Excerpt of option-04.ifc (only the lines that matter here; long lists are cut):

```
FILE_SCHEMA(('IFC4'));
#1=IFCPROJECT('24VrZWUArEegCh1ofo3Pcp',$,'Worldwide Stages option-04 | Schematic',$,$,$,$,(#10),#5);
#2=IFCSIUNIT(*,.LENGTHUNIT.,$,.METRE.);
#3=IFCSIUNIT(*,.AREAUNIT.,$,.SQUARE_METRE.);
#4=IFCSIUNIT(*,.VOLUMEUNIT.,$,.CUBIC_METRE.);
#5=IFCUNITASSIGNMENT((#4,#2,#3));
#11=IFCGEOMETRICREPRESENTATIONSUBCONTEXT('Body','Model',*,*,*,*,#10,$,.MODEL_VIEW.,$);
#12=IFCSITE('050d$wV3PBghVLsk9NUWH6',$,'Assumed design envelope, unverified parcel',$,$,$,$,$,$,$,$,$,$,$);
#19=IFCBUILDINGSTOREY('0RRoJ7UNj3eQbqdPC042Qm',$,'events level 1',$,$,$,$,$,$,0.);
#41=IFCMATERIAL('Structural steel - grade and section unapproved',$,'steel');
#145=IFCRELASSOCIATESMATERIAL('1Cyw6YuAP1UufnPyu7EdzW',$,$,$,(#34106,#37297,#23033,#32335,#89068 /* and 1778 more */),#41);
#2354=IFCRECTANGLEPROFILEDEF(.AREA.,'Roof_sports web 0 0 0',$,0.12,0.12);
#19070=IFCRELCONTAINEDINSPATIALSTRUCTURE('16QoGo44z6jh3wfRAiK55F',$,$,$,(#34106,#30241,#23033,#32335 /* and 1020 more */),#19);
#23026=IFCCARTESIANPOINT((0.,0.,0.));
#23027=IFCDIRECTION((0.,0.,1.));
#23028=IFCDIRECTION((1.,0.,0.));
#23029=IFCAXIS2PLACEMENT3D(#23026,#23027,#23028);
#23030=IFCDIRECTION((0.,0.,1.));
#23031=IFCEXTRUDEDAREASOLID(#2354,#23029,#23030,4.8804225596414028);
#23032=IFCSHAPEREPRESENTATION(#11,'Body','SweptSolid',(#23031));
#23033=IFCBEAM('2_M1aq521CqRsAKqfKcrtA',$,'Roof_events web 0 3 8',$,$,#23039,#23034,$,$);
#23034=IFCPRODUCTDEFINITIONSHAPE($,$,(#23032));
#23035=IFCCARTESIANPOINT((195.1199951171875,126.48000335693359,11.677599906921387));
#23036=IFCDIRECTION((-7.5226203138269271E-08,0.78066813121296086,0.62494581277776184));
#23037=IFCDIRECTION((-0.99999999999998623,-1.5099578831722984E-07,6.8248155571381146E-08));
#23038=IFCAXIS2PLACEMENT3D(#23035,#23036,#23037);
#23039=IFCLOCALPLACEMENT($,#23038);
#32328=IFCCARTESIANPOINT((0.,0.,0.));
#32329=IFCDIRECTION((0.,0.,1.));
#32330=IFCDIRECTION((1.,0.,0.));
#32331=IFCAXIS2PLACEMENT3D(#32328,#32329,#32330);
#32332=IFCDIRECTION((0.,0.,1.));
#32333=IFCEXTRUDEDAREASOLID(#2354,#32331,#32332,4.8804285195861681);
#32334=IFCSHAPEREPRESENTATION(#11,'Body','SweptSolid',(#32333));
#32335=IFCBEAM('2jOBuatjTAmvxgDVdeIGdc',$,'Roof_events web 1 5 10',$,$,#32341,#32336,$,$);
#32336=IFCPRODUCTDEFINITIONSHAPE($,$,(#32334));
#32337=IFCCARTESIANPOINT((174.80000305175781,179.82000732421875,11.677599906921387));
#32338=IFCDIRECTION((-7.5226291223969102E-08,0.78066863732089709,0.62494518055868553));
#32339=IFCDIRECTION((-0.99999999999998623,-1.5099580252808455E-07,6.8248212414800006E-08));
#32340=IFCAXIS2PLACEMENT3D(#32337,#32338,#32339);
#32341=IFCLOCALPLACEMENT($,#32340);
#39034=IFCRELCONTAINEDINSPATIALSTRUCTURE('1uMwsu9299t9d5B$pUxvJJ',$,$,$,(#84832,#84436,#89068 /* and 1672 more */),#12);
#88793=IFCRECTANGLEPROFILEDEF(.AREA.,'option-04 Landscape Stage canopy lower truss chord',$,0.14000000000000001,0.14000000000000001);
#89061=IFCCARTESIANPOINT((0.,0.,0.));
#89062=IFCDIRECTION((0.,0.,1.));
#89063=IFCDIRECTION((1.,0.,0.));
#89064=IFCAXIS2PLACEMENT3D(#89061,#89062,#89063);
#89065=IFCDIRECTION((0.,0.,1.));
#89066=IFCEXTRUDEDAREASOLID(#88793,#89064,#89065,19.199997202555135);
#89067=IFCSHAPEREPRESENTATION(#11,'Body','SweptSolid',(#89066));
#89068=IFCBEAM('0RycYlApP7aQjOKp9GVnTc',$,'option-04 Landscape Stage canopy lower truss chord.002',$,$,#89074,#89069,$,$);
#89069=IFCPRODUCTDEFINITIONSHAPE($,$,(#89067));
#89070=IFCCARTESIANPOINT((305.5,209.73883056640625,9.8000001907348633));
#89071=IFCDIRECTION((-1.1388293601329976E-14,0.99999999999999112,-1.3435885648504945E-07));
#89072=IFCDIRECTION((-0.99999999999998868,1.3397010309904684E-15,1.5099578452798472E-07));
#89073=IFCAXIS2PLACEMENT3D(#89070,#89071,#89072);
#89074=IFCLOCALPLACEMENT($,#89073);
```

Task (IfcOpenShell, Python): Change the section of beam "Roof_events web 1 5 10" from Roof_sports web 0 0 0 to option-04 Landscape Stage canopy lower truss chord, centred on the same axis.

```python
import ifcopenshell
import ifcopenshell.util.element
import ifcopenshell.util.representation

model = ifcopenshell.open("option-04.ifc")

member = model.by_id(32335)
source = next(p for p in model.by_type("IfcRectangleProfileDef") if p.ProfileName == "option-04 Landscape Stage canopy lower truss chord")

body = ifcopenshell.util.representation.get_representation(member, "Model", "Body")
solid = body.Items[0]
old_profile = solid.SweptArea

# Copy the section's sizes but keep this member's own profile position.
profile = ifcopenshell.util.element.copy(model, source)
profile.Position = old_profile.Position
solid.SweptArea = profile
if not model.get_total_inverses(old_profile):
    ifcopenshell.util.element.remove_deep2(model, old_profile)

print(solid.SweptArea)

model.write("option-04_rev.ifc")
```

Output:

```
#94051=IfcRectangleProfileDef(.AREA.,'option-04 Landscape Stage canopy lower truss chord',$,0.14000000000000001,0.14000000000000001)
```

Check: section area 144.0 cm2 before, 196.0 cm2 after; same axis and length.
